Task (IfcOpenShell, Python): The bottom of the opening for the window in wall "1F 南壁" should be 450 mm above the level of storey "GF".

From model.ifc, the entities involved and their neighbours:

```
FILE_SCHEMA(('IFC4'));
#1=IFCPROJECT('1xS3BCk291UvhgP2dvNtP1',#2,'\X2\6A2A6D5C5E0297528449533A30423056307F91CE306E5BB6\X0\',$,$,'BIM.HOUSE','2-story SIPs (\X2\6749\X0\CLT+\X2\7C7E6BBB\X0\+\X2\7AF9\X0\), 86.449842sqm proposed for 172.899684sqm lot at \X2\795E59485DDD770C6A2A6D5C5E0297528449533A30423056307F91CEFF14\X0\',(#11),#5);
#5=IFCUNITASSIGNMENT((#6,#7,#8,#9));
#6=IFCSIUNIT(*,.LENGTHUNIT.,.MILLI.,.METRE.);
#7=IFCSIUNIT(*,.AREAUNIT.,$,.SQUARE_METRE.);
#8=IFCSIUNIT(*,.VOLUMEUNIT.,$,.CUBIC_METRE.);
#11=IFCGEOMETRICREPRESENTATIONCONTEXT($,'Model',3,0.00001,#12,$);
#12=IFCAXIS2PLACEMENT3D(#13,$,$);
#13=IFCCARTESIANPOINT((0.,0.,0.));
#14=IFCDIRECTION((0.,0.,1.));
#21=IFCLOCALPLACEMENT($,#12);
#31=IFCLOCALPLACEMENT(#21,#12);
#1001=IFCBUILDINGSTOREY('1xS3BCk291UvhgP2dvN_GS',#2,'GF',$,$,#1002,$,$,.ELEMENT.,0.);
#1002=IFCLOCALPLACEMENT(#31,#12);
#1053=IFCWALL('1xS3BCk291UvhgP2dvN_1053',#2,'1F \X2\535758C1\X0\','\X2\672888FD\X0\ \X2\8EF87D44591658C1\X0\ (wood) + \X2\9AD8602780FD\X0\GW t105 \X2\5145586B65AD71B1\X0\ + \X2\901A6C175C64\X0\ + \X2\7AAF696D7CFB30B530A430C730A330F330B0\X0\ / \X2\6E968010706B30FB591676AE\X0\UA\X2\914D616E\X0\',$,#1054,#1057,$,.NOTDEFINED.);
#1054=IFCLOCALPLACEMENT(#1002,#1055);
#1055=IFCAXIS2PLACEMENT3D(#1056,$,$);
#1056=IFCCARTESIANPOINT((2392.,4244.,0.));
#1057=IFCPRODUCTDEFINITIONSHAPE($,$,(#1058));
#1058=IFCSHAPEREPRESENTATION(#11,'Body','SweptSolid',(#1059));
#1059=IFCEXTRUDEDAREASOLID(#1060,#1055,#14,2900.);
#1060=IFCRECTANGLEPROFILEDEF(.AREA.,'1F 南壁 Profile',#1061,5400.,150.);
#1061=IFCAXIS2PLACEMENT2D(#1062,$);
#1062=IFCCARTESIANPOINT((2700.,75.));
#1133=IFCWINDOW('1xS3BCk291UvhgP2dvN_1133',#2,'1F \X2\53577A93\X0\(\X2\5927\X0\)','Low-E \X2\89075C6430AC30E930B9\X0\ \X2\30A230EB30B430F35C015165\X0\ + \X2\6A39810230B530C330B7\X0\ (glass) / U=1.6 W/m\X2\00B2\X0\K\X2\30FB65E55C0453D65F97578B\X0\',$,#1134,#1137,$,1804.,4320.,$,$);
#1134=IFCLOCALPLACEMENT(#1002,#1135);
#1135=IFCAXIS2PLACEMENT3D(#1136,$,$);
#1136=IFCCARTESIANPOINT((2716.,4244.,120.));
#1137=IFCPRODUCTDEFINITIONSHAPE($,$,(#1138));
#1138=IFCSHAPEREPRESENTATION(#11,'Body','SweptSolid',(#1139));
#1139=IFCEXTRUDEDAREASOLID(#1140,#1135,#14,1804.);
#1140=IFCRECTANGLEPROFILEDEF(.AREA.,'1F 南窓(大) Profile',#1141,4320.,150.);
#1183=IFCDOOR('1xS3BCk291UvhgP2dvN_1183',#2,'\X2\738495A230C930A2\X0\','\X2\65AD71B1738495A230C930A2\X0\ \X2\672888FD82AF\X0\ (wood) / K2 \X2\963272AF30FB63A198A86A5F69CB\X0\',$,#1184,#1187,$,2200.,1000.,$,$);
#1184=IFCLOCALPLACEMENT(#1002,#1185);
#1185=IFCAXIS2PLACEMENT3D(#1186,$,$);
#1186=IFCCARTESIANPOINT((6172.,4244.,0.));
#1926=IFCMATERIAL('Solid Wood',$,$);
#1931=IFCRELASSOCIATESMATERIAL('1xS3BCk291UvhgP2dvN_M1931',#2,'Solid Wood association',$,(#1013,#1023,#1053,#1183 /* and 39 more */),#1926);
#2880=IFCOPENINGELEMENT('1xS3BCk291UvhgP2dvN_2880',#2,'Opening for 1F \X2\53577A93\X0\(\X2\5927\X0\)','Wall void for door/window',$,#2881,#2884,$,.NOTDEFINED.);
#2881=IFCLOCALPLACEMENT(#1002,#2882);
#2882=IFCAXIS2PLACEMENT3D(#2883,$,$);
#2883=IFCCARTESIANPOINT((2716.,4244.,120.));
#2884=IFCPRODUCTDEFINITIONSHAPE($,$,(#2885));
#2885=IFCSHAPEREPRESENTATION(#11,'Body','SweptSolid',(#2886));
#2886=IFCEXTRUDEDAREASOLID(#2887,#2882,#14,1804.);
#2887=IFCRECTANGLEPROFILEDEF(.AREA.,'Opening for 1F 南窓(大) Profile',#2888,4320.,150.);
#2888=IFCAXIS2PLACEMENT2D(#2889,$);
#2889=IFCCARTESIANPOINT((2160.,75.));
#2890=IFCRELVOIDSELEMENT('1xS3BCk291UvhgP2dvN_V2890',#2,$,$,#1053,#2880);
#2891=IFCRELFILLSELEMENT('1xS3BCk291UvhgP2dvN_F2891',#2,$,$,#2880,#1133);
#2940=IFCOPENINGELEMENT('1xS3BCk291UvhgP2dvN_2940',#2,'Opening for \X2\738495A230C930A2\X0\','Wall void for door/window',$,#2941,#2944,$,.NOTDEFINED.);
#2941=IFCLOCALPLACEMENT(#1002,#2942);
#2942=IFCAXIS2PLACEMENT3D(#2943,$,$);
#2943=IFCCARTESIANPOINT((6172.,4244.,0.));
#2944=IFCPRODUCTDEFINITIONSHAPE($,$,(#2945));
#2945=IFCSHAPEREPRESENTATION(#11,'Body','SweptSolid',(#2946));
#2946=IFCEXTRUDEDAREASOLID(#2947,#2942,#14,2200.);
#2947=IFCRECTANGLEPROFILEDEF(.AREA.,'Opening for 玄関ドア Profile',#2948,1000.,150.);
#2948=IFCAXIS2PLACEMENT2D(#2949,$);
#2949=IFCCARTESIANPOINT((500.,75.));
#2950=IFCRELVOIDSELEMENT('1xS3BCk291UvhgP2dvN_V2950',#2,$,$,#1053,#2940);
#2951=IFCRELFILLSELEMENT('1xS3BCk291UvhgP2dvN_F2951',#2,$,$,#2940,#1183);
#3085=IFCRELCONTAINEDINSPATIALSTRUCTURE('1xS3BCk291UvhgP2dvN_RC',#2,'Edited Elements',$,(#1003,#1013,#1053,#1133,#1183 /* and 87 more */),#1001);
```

```python
import numpy as np
import ifcopenshell
import ifcopenshell.api.geometry
import ifcopenshell.geom
import ifcopenshell.util.element
import ifcopenshell.util.placement
import ifcopenshell.util.shape
import ifcopenshell.util.unit

model = ifcopenshell.open("model.ifc")
unit_scale = ifcopenshell.util.unit.calculate_unit_scale(model)

window = model.by_guid("1xS3BCk291UvhgP2dvN_1133")
opening = window.FillsVoids[0].RelatingOpeningElement
storey = ifcopenshell.util.element.get_container(window, ifc_class="IfcBuildingStorey")
level = ifcopenshell.util.placement.get_local_placement(storey.ObjectPlacement)[2, 3]

# The opening's origin need not be at the sill, so measure its lowest point.
shape = ifcopenshell.geom.create_shape(ifcopenshell.geom.settings(), opening)
bottom = ifcopenshell.util.shape.get_shape_bottom_elevation(shape, shape.geometry) / unit_scale
dz = level + 450.0 - bottom

shift = np.array([0.0, 0.0, dz])
# The window is not placed relative to its opening, so move both.
for product in (opening, window):
    matrix = ifcopenshell.util.placement.get_local_placement(product.ObjectPlacement)
    matrix[:3, 3] += shift
    ifcopenshell.api.geometry.edit_object_placement(model, product=product, matrix=matrix, is_si=False)

print(f"moved by {dz * unit_scale:+.3f} m")

model.write("model_edited.ifc")
```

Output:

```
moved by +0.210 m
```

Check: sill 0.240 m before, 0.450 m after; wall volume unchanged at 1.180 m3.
